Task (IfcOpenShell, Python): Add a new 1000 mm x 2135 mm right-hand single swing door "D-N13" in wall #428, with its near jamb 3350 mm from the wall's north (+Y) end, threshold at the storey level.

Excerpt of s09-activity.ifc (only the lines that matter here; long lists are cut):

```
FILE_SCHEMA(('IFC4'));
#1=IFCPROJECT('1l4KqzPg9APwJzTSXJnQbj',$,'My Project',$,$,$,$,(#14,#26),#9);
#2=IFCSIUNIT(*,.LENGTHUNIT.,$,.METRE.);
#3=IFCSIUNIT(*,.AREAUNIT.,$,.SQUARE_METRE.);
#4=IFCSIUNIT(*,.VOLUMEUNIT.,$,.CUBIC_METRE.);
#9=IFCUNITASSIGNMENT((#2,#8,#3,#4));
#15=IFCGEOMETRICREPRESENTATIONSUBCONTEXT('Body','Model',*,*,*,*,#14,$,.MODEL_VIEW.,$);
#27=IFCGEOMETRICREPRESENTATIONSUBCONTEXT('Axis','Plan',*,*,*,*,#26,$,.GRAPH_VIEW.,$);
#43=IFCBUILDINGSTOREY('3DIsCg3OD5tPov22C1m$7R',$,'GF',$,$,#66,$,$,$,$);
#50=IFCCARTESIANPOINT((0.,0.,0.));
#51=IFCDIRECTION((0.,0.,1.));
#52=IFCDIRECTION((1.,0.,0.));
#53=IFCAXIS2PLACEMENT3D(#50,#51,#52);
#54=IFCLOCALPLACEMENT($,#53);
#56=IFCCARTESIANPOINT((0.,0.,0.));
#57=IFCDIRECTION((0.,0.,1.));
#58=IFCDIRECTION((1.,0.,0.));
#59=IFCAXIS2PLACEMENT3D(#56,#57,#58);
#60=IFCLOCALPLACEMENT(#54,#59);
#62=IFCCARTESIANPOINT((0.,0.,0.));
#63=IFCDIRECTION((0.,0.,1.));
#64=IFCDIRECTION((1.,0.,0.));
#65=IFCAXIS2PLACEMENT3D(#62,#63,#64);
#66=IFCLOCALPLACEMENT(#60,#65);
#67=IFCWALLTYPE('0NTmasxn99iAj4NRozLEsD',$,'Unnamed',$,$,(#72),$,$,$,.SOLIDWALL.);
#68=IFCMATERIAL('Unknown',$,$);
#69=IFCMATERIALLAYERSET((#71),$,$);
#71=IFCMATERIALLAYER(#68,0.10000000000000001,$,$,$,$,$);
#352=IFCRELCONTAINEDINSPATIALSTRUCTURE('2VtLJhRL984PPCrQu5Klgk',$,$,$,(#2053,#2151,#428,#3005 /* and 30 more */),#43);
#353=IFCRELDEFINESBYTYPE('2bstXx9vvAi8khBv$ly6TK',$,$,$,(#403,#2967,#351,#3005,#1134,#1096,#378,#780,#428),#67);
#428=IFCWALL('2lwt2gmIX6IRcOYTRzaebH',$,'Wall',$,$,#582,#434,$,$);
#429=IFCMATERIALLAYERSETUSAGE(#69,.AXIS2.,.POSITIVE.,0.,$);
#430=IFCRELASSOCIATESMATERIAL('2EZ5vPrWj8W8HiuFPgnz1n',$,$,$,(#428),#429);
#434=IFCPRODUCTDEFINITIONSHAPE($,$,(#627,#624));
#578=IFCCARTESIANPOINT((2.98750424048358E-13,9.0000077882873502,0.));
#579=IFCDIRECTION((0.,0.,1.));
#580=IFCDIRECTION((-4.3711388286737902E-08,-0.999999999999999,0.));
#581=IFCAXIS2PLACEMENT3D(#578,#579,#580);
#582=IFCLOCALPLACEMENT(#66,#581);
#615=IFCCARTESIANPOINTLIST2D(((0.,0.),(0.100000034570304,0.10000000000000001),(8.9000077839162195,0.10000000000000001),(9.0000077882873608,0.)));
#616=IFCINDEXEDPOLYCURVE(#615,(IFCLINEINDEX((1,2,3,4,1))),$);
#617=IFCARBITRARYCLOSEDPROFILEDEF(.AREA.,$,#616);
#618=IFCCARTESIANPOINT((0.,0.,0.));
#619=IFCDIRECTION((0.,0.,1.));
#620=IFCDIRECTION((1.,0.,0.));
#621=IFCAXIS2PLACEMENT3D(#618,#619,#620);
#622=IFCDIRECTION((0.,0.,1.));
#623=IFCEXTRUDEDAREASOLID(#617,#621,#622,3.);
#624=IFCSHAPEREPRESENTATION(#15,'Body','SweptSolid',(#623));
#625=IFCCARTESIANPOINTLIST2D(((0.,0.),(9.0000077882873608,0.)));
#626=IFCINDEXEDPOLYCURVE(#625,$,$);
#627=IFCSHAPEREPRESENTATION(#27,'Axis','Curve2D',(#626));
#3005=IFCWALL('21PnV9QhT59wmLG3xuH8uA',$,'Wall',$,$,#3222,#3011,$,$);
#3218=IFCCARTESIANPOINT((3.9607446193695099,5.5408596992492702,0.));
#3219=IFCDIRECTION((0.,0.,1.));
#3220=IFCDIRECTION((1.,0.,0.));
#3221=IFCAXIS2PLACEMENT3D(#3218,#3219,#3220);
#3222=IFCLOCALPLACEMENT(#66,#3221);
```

```python
import numpy as np
import ifcopenshell
import ifcopenshell.api.feature
import ifcopenshell.api.geometry
import ifcopenshell.api.root
import ifcopenshell.api.spatial
import ifcopenshell.geom
import ifcopenshell.util.element
import ifcopenshell.util.placement
import ifcopenshell.util.representation
import ifcopenshell.util.shape
import ifcopenshell.util.unit

model = ifcopenshell.open("s09-activity.ifc")
unit_scale = ifcopenshell.util.unit.calculate_unit_scale(model)
settings = ifcopenshell.geom.settings()


def volume(element):
    """Net volume in cubic metres, openings subtracted."""
    shape = ifcopenshell.geom.create_shape(settings, element)
    return ifcopenshell.util.shape.get_volume(shape.geometry)


wall = model.by_id(428)
storey = ifcopenshell.util.element.get_container(wall, ifc_class="IfcBuildingStorey")
context = ifcopenshell.util.representation.get_context(model, "Model", "Body", "MODEL_VIEW")
before = volume(wall)

width, height, from_end, sill = 1, 2.135, 3.35, 0.0  # metres

# The wall runs along its own X axis, and the end named is its -X end.
wall_shape = ifcopenshell.geom.create_shape(settings, wall)
x, y, z = ifcopenshell.util.shape.get_vertices(wall_shape.geometry).T
start = x.min() + from_end
face, thickness = float(y.min()), float(y.max() - y.min())
wall_matrix = ifcopenshell.util.placement.get_local_placement(wall.ObjectPlacement)
level = ifcopenshell.util.placement.get_local_placement(storey.ObjectPlacement)[2, 3]


def in_wall(x, y):
    """Placement at x, y metres in the wall's axes, at sill height."""
    matrix = wall_matrix.copy()
    matrix[:, 3] = wall_matrix @ np.array([x / unit_scale, y / unit_scale, 0.0, 1.0])
    matrix[2, 3] = level + sill / unit_scale
    return matrix


# Opening: a box that overshoots both wall faces by 50 mm.
opening = ifcopenshell.api.root.create_entity(model, ifc_class="IfcOpeningElement", predefined_type="OPENING")
box = ifcopenshell.api.geometry.add_wall_representation(
    model, context=context, length=width, height=height, thickness=thickness + 0.1
)
ifcopenshell.api.geometry.assign_representation(model, product=opening, representation=box)
ifcopenshell.api.geometry.edit_object_placement(model, product=opening, matrix=in_wall(start, face - 0.05), is_si=False)
ifcopenshell.api.feature.add_feature(model, feature=opening, element=wall)

door = ifcopenshell.api.root.create_entity(model, ifc_class="IfcDoor", name="D-N13", predefined_type="DOOR")
door.OverallWidth, door.OverallHeight = width / unit_scale, height / unit_scale
door.OperationType = "SINGLE_SWING_RIGHT"
body = ifcopenshell.api.geometry.add_door_representation(
    model,
    context=context,
    overall_width=door.OverallWidth,
    overall_height=door.OverallHeight,
    operation_type="SINGLE_SWING_RIGHT",
    lining_properties={"LiningDepth": thickness / unit_scale, "ThresholdDepth": thickness / unit_scale},
)
ifcopenshell.api.geometry.assign_representation(model, product=door, representation=body)
ifcopenshell.api.spatial.assign_container(model, products=[door], relating_structure=storey)
ifcopenshell.api.feature.add_filling(model, opening=opening, element=door)

# The lining spans the wall, so the door starts at the wall face.
ifcopenshell.api.geometry.edit_object_placement(model, product=door, matrix=in_wall(start, face), is_si=False)

after = volume(wall)

print(f"wall volume {before:.3f} -> {after:.3f} m3")

model.write("s09-activity-out.ifc")
```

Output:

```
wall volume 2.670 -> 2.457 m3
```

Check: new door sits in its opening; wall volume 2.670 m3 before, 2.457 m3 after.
